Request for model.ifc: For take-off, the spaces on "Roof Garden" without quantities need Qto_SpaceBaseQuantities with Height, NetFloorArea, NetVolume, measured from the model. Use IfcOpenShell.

First a look at what the model holds.

```python
import ifcopenshell
import ifcopenshell.util.element
import ifcopenshell.util.unit

model = ifcopenshell.open("model.ifc")
print(model.schema)
for unit_type in ("LENGTHUNIT", "AREAUNIT", "VOLUMEUNIT"):
    print(unit_type, ifcopenshell.util.unit.calculate_unit_scale(model, unit_type))
storey = next(s for s in model.by_type("IfcBuildingStorey") if s.Name == "Roof Garden")
spaces = [e for e in ifcopenshell.util.element.get_decomposition(storey) if e.is_a("IfcSpace")]
for e in sorted(spaces, key=lambda e: e.id()):
    print(e.id(), e.is_a(), e.Name, list(ifcopenshell.util.element.get_psets(e, qtos_only=True)), sep=" | ")
```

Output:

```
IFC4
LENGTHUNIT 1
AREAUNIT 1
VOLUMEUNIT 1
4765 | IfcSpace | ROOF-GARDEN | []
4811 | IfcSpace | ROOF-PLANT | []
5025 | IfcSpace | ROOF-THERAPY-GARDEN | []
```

```python
import ifcopenshell
import ifcopenshell.api.pset
import ifcopenshell.geom
import ifcopenshell.util.element
import ifcopenshell.util.shape
import ifcopenshell.util.unit

model = ifcopenshell.open("model.ifc")
unit_scale = ifcopenshell.util.unit.calculate_unit_scale(model)
area_scale = ifcopenshell.util.unit.calculate_unit_scale(model, "AREAUNIT")
volume_scale = ifcopenshell.util.unit.calculate_unit_scale(model, "VOLUMEUNIT")
settings = ifcopenshell.geom.settings()

storey = next(s for s in model.by_type("IfcBuildingStorey") if s.Name == "Roof Garden")
spaces = [e for e in ifcopenshell.util.element.get_decomposition(storey) if e.is_a("IfcSpace")]

for e in sorted(spaces, key=lambda e: e.id()):
    if ifcopenshell.util.element.get_psets(e, qtos_only=True, should_inherit=False):
        continue
    # Geometry comes back in metres, in the element's own axes.
    shape = ifcopenshell.geom.create_shape(settings, e)
    values = {
        "Height": ifcopenshell.util.shape.get_z(shape.geometry) / unit_scale,
        "NetFloorArea": ifcopenshell.util.shape.get_footprint_area(shape.geometry) / area_scale,
        "NetVolume": ifcopenshell.util.shape.get_volume(shape.geometry) / volume_scale,
    }
    qto = ifcopenshell.api.pset.add_qto(model, product=e, name="Qto_SpaceBaseQuantities")
    ifcopenshell.api.pset.edit_qto(model, qto=qto, properties=values)
    print(e.id(), {k: round(v, 3) for k, v in values.items()})

model.write("model_edited.ifc")
```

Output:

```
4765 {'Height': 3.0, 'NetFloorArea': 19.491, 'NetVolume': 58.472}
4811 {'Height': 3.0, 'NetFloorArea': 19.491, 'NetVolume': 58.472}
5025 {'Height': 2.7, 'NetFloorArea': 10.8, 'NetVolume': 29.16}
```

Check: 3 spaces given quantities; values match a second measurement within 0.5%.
